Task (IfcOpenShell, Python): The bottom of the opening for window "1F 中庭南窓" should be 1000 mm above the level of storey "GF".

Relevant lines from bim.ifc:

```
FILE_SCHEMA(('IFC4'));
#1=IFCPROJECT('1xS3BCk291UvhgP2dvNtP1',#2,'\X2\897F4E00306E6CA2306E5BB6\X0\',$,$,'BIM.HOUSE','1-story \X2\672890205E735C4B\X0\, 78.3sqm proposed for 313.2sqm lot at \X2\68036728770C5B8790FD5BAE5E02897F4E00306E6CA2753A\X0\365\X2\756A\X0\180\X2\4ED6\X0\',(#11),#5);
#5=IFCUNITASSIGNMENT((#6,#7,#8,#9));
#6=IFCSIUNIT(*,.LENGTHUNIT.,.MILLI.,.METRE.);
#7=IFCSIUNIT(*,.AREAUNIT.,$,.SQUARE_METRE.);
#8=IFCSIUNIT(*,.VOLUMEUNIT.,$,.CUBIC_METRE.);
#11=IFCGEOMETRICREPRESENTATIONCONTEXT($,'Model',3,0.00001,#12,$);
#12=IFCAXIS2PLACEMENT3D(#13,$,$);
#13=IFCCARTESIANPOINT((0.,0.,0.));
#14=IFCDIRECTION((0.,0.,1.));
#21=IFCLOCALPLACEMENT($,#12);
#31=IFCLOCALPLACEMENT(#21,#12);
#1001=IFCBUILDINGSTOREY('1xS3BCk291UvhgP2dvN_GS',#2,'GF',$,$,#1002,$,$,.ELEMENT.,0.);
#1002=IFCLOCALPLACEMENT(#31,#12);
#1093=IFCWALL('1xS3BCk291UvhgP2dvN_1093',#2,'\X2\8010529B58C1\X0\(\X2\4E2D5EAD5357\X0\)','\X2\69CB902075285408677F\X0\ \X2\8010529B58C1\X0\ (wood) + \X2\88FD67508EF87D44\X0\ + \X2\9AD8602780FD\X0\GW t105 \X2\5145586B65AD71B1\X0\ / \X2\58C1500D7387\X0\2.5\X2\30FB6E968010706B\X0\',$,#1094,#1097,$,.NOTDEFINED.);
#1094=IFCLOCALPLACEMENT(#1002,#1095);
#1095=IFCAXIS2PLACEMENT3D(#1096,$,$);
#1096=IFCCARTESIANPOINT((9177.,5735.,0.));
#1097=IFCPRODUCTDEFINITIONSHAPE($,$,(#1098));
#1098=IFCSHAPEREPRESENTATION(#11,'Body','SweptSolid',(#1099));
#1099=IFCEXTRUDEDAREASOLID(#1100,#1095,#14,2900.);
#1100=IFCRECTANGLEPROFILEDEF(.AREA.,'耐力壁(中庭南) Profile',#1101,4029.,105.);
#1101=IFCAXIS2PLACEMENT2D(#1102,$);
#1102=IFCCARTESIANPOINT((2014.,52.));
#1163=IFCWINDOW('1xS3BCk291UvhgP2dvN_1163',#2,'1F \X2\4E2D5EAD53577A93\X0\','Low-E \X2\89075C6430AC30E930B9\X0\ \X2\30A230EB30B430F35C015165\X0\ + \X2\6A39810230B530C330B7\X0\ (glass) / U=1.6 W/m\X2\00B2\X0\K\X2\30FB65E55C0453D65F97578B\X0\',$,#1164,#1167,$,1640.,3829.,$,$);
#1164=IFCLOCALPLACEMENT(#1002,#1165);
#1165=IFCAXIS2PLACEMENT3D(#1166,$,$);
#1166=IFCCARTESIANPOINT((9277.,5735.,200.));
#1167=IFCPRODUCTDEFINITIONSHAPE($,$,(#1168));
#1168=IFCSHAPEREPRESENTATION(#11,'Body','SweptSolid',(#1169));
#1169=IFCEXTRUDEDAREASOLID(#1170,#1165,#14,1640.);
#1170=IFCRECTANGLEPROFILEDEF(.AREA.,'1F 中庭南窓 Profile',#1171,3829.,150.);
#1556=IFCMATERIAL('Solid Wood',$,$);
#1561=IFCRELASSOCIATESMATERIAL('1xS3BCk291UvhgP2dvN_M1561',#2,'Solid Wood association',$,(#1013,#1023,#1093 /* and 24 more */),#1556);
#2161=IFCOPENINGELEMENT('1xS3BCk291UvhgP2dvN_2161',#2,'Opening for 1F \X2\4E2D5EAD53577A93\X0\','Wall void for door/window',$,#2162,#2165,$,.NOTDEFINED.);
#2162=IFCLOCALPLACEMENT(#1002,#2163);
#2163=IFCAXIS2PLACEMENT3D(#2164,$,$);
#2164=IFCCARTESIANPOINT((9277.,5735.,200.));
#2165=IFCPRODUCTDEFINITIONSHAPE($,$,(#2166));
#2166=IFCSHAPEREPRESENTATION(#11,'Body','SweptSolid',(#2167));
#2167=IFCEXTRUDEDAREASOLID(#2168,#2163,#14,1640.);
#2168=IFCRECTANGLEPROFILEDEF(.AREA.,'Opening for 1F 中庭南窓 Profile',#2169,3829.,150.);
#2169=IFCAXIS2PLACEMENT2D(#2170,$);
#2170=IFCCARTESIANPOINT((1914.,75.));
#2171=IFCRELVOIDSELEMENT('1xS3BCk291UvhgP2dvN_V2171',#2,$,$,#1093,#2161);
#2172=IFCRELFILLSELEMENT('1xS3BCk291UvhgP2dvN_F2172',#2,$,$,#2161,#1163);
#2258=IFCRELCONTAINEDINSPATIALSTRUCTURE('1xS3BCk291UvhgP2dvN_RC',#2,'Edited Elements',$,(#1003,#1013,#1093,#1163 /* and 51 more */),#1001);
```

```python
import numpy as np
import ifcopenshell
import ifcopenshell.api.geometry
import ifcopenshell.geom
import ifcopenshell.util.element
import ifcopenshell.util.placement
import ifcopenshell.util.shape
import ifcopenshell.util.unit

model = ifcopenshell.open("bim.ifc")
unit_scale = ifcopenshell.util.unit.calculate_unit_scale(model)

window = model.by_guid("1xS3BCk291UvhgP2dvN_1163")
opening = window.FillsVoids[0].RelatingOpeningElement
storey = ifcopenshell.util.element.get_container(window, ifc_class="IfcBuildingStorey")
level = ifcopenshell.util.placement.get_local_placement(storey.ObjectPlacement)[2, 3]

# The opening's origin need not be at the sill, so measure its lowest point.
shape = ifcopenshell.geom.create_shape(ifcopenshell.geom.settings(), opening)
bottom = ifcopenshell.util.shape.get_shape_bottom_elevation(shape, shape.geometry) / unit_scale
dz = level + 1000.0 - bottom

shift = np.array([0.0, 0.0, dz])
# The window is not placed relative to its opening, so move both.
for product in (opening, window):
    matrix = ifcopenshell.util.placement.get_local_placement(product.ObjectPlacement)
    matrix[:3, 3] += shift
    ifcopenshell.api.geometry.edit_object_placement(model, product=product, matrix=matrix, is_si=False)

print(f"moved by {dz * unit_scale:+.3f} m")

model.write("bim_v2.ifc")
```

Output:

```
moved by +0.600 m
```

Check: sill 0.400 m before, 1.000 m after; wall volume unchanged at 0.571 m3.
